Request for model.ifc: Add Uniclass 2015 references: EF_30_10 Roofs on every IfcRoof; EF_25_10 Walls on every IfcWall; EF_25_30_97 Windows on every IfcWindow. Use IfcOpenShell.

First a look at what the model holds.

```python
import ifcopenshell

model = ifcopenshell.open("model.ifc")
print(model.schema)
print("classifications:", [c.Name for c in model.by_type("IfcClassification")])
for ifc_class in ("IfcDoor", "IfcRoof", "IfcStair", "IfcWall", "IfcWindow"):
    print(ifc_class, len(model.by_type(ifc_class)))
```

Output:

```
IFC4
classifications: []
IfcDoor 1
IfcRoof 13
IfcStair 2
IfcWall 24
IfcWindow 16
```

```python
import ifcopenshell
import ifcopenshell.api.classification

model = ifcopenshell.open("model.ifc")

system = ifcopenshell.api.classification.add_classification(model, classification="Uniclass 2015")

codes = {
    "IfcRoof": ("EF_30_10", "Roofs"),
    "IfcWall": ("EF_25_10", "Walls"),
    "IfcWindow": ("EF_25_30_97", "Windows"),
}
for ifc_class, (code, name) in codes.items():
    products = model.by_type(ifc_class)
    ifcopenshell.api.classification.add_reference(
        model, products=products, classification=system, identification=code, name=name
    )
    print(code, len(products))

model.write("model_edited.ifc")
```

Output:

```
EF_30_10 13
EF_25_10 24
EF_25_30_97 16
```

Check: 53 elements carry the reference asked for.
